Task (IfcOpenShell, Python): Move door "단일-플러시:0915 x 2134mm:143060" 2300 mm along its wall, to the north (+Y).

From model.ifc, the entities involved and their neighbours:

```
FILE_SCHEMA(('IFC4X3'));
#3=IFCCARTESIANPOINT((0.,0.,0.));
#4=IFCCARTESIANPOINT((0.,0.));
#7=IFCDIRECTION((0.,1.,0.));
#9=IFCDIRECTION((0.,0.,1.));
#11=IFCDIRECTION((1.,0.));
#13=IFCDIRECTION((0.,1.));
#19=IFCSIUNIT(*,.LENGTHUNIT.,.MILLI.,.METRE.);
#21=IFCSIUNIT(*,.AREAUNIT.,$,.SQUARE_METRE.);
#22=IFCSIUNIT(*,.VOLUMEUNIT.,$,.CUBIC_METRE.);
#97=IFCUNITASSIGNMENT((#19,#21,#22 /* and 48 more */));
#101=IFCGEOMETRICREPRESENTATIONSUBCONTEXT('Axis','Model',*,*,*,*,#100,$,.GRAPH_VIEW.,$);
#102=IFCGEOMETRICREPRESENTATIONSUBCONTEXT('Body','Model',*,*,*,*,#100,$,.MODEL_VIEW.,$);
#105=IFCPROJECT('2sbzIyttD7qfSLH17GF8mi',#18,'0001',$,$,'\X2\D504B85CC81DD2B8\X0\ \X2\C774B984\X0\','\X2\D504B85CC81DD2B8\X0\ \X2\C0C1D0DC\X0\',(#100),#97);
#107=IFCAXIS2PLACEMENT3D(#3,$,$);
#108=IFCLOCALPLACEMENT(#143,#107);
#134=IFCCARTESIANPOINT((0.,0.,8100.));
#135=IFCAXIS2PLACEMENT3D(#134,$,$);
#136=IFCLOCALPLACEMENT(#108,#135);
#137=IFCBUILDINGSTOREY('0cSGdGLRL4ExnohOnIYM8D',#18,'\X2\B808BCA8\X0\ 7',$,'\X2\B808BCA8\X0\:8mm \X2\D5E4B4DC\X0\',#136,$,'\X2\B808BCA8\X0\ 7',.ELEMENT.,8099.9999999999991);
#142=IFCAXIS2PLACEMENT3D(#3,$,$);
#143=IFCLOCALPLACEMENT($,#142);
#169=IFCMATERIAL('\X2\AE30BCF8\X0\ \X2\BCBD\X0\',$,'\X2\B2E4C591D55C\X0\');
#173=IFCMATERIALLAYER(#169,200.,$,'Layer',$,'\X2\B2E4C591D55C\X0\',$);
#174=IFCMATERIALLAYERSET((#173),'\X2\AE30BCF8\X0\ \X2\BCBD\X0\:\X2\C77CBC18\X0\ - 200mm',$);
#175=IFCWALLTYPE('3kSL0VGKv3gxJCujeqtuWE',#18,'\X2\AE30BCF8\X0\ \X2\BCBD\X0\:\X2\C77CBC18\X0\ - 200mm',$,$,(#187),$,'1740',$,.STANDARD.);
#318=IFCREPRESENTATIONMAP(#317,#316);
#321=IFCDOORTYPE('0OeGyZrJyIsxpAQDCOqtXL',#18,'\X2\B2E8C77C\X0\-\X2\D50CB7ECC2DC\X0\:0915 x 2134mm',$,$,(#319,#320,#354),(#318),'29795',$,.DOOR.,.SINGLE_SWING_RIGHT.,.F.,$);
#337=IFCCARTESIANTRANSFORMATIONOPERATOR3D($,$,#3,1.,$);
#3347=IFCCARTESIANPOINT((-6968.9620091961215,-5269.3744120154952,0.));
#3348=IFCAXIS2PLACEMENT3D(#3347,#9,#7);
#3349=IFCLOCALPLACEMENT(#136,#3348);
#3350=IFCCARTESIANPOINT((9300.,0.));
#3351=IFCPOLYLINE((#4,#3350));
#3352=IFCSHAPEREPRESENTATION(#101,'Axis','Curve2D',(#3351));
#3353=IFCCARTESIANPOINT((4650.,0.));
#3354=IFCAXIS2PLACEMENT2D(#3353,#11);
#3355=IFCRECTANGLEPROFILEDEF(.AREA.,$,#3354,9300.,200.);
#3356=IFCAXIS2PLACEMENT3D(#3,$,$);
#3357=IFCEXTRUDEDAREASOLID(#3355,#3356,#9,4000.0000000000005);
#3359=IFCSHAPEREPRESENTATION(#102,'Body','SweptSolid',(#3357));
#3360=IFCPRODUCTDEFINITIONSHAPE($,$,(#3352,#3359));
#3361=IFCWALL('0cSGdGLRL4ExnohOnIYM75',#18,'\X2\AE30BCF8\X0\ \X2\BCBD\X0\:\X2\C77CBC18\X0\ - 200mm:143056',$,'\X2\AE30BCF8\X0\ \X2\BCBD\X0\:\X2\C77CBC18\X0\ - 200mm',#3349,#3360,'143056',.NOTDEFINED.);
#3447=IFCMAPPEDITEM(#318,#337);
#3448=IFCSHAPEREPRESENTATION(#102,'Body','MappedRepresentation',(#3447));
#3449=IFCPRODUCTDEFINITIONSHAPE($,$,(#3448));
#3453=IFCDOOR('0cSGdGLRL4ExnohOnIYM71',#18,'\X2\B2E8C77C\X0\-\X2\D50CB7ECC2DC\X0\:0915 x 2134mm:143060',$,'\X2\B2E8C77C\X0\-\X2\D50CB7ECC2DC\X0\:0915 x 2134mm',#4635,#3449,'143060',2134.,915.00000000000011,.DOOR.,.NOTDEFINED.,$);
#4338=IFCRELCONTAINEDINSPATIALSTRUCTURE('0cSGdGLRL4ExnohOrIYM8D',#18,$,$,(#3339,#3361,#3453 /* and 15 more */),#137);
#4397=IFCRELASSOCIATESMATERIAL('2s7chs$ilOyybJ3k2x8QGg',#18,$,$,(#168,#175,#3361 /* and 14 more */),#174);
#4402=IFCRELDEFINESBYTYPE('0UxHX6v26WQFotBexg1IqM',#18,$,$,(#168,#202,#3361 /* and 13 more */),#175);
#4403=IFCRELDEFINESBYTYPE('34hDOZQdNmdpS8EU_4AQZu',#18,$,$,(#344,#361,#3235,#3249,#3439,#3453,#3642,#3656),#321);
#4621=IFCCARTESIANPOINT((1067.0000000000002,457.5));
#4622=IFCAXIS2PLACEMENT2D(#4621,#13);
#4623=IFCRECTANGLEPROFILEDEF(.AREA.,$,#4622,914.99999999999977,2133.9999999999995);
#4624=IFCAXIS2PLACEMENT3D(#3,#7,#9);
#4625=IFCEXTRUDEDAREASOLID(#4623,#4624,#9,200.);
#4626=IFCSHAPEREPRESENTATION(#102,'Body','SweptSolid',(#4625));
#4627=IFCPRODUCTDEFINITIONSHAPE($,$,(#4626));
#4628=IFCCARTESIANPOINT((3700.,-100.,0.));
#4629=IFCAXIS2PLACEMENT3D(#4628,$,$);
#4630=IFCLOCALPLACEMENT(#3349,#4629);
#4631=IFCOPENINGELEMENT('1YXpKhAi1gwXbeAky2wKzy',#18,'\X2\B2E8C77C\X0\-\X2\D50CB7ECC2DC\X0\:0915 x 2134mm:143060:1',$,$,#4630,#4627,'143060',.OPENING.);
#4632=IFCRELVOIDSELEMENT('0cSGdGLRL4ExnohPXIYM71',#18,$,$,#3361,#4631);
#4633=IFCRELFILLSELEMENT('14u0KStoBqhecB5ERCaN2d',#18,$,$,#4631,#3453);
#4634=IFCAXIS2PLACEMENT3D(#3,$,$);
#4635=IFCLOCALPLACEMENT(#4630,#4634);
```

```python
import ifcopenshell
import ifcopenshell.api.geometry
import ifcopenshell.util.placement
import ifcopenshell.util.unit

model = ifcopenshell.open("model.ifc")
unit_scale = ifcopenshell.util.unit.calculate_unit_scale(model)

door = model.by_guid("0cSGdGLRL4ExnohOnIYM71")
opening = door.FillsVoids[0].RelatingOpeningElement
wall = opening.VoidsElements[0].RelatingBuildingElement

wall_matrix = ifcopenshell.util.placement.get_local_placement(wall.ObjectPlacement)
shift = wall_matrix[:3, 0] * 2.3 / unit_scale
before = ifcopenshell.util.placement.get_local_placement(door.ObjectPlacement)[:3, 3].copy()

# The door is placed relative to its opening, so it follows when the opening moves.
matrix = ifcopenshell.util.placement.get_local_placement(opening.ObjectPlacement)
matrix[:3, 3] += shift
ifcopenshell.api.geometry.edit_object_placement(
    model, product=opening, matrix=matrix, is_si=False, should_transform_children=True
)

after = ifcopenshell.util.placement.get_local_placement(door.ObjectPlacement)[:3, 3]
print("door moved by", (after - before).round(3) + 0.0)

model.write("model_updated.ifc")
```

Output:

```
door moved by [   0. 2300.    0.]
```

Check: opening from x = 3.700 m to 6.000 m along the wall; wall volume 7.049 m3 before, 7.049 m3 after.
